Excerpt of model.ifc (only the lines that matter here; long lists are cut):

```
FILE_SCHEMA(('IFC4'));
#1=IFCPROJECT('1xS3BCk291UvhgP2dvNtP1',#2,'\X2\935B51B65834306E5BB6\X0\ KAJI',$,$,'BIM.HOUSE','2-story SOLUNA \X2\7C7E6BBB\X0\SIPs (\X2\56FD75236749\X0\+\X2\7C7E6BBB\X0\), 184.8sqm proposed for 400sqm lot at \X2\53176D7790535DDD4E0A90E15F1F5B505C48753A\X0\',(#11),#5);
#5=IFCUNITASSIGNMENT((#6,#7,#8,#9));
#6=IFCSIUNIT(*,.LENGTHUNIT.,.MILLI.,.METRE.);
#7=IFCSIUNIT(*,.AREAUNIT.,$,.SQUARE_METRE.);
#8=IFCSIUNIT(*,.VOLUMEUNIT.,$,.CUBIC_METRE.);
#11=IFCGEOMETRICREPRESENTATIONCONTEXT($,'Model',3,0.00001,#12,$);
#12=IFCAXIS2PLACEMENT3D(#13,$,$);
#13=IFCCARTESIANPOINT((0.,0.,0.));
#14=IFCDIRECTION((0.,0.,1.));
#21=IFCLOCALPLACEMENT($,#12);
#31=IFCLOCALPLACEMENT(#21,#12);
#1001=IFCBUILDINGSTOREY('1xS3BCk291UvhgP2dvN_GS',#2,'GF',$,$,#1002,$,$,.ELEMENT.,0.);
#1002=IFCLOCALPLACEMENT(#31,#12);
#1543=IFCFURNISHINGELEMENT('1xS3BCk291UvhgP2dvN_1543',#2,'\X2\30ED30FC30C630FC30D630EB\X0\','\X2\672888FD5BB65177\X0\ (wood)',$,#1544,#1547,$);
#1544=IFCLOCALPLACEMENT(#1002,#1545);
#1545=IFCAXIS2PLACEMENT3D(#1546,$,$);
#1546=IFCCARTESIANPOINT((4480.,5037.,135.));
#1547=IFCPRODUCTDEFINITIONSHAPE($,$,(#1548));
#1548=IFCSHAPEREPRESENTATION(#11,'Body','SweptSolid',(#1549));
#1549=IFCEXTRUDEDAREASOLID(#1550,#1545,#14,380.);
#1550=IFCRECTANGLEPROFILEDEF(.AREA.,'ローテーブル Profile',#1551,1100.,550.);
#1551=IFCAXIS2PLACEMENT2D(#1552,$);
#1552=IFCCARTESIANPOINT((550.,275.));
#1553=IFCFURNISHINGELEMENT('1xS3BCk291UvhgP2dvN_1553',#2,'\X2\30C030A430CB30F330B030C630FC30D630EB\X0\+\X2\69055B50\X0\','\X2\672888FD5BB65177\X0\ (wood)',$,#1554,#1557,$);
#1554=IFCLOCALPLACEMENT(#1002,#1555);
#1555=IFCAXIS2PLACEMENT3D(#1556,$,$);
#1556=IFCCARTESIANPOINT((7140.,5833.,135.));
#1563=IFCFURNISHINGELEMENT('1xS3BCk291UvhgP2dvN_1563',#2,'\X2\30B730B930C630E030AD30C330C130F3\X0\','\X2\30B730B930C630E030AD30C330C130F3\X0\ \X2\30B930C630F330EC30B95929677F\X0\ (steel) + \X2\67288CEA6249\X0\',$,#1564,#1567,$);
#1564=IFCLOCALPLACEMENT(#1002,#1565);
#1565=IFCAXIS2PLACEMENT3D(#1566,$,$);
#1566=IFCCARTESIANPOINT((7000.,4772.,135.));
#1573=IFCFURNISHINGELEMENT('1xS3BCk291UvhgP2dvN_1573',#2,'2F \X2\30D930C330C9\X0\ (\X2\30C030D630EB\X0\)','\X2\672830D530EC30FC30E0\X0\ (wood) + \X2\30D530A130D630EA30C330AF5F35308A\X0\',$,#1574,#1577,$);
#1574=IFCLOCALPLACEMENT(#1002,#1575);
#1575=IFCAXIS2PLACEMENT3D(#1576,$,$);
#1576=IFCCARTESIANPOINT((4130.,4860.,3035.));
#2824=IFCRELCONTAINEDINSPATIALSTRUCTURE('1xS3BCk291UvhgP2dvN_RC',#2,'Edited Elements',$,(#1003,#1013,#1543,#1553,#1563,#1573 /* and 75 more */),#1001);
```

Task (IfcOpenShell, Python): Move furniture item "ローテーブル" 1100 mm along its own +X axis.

```python
import ifcopenshell
import ifcopenshell.api.geometry
import ifcopenshell.util.placement
import ifcopenshell.util.unit

model = ifcopenshell.open("model.ifc")
unit_scale = ifcopenshell.util.unit.calculate_unit_scale(model)

item = model.by_id(1543)
matrix = ifcopenshell.util.placement.get_local_placement(item.ObjectPlacement)
matrix[:3, 3] += matrix[:3, 0] * 1.1 / unit_scale
ifcopenshell.api.geometry.edit_object_placement(model, product=item, matrix=matrix, is_si=False)

print(ifcopenshell.util.placement.get_local_placement(item.ObjectPlacement).round(3) + 0.0)

model.write("model_edited.ifc")
```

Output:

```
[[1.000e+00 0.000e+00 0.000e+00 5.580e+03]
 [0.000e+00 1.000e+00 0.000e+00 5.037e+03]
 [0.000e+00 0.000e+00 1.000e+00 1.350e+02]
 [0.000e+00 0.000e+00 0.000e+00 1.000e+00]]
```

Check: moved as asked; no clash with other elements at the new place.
